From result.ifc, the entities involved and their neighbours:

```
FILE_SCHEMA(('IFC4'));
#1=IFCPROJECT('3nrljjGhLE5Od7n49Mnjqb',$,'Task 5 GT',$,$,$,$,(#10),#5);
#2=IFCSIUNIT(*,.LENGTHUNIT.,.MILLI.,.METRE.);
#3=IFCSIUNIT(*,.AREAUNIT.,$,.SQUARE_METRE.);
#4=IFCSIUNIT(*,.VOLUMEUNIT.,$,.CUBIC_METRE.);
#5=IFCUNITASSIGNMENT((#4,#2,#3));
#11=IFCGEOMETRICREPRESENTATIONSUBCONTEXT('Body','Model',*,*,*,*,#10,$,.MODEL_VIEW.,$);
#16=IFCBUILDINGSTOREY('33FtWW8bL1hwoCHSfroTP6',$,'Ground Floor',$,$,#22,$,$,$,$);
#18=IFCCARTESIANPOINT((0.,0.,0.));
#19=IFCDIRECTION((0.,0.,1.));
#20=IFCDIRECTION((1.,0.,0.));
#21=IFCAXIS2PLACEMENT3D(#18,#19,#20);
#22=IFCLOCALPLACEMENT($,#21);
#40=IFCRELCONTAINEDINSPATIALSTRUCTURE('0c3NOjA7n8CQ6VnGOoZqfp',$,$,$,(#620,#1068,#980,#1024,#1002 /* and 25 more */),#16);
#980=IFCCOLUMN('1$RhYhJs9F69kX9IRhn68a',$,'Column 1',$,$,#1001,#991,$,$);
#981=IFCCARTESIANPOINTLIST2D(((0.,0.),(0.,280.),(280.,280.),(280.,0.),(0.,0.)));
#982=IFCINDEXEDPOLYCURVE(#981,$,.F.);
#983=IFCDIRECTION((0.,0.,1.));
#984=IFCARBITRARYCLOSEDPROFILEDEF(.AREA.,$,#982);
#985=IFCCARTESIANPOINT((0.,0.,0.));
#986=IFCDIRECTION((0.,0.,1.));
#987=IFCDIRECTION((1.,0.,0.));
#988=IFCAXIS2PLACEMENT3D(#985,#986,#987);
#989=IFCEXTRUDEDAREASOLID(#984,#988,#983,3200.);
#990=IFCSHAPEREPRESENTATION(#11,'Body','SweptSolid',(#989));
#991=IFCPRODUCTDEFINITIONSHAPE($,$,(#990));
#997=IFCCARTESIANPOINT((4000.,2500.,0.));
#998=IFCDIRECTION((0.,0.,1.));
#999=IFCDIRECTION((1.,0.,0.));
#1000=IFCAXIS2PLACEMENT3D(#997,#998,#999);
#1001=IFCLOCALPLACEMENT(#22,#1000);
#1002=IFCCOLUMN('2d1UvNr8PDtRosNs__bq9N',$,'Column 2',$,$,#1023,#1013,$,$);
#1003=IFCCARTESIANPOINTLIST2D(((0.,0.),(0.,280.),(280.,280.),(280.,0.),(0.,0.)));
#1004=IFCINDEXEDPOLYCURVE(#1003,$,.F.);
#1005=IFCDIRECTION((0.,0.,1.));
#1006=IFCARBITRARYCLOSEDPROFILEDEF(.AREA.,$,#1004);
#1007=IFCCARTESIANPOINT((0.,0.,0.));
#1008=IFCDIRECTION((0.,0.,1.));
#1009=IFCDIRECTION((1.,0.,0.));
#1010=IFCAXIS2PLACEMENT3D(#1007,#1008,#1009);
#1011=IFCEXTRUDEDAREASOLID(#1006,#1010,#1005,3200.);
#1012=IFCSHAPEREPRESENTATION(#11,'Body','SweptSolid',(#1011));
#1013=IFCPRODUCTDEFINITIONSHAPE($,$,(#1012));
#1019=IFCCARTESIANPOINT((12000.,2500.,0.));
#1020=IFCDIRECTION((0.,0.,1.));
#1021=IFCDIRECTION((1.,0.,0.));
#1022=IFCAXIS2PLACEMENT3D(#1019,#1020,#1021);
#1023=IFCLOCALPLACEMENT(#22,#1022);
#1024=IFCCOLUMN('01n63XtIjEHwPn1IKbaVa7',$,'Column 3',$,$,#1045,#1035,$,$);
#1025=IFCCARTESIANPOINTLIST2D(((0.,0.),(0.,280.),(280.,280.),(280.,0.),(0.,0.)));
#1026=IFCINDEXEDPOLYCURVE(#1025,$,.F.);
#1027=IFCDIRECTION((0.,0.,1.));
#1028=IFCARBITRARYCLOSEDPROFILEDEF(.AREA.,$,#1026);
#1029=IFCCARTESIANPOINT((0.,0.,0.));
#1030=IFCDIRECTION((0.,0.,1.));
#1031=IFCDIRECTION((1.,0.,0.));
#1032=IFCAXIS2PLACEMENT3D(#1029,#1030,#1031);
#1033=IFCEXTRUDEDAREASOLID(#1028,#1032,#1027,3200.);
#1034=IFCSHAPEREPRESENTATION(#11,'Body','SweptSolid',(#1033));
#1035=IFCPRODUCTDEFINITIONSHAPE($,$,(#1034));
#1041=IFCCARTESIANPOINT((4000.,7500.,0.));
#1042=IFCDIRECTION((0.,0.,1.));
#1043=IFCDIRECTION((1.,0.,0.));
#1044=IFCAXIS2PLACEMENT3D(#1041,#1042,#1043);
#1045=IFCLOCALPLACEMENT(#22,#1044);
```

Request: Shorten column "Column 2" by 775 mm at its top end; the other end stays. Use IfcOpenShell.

```python
import ifcopenshell
import ifcopenshell.util.representation
import ifcopenshell.util.unit

model = ifcopenshell.open("result.ifc")
unit_scale = ifcopenshell.util.unit.calculate_unit_scale(model)

member = model.by_id(1002)
change = -0.775 / unit_scale

# The extrusion runs towards the end named, so only its depth changes.
body = ifcopenshell.util.representation.get_representation(member, "Model", "Body")
solid = body.Items[0]
old_length = solid.Depth
solid.Depth += change

print(f"length {old_length:g} -> {solid.Depth:g}")

model.write("result_updated.ifc")
```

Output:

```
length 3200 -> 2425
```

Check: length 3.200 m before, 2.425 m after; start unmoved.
